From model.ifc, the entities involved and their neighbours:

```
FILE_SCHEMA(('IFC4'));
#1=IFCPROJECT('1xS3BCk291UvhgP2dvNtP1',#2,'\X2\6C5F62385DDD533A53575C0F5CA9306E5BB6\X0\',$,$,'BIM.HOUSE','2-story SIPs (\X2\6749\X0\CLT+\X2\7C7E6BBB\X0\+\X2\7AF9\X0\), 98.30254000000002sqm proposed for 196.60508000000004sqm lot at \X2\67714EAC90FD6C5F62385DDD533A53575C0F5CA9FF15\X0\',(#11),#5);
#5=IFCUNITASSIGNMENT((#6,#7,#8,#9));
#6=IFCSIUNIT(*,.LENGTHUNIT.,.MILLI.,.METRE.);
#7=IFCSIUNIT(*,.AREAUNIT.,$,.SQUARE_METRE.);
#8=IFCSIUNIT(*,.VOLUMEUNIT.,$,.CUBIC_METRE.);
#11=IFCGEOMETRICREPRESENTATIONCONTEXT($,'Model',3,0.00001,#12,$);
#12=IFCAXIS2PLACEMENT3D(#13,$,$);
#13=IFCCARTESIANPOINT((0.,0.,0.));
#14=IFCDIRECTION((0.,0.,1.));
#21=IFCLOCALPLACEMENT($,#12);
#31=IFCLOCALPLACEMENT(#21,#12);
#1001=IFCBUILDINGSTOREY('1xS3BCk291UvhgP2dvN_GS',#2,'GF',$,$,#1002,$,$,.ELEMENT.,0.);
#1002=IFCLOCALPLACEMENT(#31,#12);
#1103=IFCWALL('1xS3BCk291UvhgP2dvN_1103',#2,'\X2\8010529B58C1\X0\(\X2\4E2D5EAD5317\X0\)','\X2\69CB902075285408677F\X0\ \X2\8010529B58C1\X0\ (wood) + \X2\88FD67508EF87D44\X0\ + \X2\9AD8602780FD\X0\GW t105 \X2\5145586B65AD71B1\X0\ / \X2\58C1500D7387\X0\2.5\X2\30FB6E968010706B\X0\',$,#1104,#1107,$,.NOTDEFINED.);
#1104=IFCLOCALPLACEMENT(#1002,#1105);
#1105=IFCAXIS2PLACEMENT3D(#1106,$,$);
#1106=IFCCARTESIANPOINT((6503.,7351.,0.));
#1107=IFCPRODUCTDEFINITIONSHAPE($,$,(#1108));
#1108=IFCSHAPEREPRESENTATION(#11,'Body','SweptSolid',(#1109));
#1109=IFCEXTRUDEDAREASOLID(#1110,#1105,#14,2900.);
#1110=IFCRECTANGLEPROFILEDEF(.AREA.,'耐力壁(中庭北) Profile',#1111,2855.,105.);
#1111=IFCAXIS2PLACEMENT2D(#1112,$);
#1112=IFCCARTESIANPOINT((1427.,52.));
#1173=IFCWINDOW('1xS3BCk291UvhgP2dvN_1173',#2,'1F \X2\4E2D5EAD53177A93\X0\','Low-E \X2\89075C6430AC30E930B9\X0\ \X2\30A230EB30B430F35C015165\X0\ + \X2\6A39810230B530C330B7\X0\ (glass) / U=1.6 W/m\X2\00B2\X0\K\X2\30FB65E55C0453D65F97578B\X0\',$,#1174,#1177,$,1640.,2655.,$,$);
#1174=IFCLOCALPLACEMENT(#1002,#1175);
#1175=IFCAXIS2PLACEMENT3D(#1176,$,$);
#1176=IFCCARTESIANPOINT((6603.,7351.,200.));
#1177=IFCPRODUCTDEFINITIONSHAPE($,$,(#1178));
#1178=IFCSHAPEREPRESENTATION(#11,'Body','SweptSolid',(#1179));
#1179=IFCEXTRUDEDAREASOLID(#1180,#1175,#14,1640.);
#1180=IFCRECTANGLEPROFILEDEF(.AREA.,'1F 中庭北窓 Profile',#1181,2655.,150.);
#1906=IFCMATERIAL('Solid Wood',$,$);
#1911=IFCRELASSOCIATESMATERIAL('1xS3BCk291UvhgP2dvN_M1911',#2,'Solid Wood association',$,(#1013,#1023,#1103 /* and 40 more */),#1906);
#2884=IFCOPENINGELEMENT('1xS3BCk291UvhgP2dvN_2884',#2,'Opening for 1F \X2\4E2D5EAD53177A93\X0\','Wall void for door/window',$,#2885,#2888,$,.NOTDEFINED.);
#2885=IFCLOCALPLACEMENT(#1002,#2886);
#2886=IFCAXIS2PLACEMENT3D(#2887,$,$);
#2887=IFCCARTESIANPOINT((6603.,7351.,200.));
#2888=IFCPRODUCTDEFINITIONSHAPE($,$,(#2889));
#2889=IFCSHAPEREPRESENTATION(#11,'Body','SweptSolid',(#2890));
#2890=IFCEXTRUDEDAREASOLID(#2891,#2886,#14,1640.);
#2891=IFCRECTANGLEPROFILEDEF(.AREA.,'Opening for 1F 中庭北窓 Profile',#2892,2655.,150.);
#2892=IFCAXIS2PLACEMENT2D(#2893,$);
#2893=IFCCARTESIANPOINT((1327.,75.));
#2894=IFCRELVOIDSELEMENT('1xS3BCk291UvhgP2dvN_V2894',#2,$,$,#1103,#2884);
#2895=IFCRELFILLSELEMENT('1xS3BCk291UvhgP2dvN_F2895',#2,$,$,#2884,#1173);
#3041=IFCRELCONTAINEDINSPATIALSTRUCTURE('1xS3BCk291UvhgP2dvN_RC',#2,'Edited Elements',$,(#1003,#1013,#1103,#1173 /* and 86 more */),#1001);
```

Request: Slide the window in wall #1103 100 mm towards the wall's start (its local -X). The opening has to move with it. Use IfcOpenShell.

```python
import ifcopenshell
import ifcopenshell.api.geometry
import ifcopenshell.util.placement
import ifcopenshell.util.unit

model = ifcopenshell.open("model.ifc")
unit_scale = ifcopenshell.util.unit.calculate_unit_scale(model)

window = model.by_guid("1xS3BCk291UvhgP2dvN_1173")
opening = window.FillsVoids[0].RelatingOpeningElement
wall = opening.VoidsElements[0].RelatingBuildingElement

wall_matrix = ifcopenshell.util.placement.get_local_placement(wall.ObjectPlacement)
shift = wall_matrix[:3, 0] * -0.1 / unit_scale
before = ifcopenshell.util.placement.get_local_placement(window.ObjectPlacement)[:3, 3].copy()

# The window is not placed relative to its opening, so move both.
for product in (opening, window):
    matrix = ifcopenshell.util.placement.get_local_placement(product.ObjectPlacement)
    matrix[:3, 3] += shift
    ifcopenshell.api.geometry.edit_object_placement(model, product=product, matrix=matrix, is_si=False)

after = ifcopenshell.util.placement.get_local_placement(window.ObjectPlacement)[:3, 3]
print("window moved by", (after - before).round(3) + 0.0)

model.write("model_edited.ifc")
```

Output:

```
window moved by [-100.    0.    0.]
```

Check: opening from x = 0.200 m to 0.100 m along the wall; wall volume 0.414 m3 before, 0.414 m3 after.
